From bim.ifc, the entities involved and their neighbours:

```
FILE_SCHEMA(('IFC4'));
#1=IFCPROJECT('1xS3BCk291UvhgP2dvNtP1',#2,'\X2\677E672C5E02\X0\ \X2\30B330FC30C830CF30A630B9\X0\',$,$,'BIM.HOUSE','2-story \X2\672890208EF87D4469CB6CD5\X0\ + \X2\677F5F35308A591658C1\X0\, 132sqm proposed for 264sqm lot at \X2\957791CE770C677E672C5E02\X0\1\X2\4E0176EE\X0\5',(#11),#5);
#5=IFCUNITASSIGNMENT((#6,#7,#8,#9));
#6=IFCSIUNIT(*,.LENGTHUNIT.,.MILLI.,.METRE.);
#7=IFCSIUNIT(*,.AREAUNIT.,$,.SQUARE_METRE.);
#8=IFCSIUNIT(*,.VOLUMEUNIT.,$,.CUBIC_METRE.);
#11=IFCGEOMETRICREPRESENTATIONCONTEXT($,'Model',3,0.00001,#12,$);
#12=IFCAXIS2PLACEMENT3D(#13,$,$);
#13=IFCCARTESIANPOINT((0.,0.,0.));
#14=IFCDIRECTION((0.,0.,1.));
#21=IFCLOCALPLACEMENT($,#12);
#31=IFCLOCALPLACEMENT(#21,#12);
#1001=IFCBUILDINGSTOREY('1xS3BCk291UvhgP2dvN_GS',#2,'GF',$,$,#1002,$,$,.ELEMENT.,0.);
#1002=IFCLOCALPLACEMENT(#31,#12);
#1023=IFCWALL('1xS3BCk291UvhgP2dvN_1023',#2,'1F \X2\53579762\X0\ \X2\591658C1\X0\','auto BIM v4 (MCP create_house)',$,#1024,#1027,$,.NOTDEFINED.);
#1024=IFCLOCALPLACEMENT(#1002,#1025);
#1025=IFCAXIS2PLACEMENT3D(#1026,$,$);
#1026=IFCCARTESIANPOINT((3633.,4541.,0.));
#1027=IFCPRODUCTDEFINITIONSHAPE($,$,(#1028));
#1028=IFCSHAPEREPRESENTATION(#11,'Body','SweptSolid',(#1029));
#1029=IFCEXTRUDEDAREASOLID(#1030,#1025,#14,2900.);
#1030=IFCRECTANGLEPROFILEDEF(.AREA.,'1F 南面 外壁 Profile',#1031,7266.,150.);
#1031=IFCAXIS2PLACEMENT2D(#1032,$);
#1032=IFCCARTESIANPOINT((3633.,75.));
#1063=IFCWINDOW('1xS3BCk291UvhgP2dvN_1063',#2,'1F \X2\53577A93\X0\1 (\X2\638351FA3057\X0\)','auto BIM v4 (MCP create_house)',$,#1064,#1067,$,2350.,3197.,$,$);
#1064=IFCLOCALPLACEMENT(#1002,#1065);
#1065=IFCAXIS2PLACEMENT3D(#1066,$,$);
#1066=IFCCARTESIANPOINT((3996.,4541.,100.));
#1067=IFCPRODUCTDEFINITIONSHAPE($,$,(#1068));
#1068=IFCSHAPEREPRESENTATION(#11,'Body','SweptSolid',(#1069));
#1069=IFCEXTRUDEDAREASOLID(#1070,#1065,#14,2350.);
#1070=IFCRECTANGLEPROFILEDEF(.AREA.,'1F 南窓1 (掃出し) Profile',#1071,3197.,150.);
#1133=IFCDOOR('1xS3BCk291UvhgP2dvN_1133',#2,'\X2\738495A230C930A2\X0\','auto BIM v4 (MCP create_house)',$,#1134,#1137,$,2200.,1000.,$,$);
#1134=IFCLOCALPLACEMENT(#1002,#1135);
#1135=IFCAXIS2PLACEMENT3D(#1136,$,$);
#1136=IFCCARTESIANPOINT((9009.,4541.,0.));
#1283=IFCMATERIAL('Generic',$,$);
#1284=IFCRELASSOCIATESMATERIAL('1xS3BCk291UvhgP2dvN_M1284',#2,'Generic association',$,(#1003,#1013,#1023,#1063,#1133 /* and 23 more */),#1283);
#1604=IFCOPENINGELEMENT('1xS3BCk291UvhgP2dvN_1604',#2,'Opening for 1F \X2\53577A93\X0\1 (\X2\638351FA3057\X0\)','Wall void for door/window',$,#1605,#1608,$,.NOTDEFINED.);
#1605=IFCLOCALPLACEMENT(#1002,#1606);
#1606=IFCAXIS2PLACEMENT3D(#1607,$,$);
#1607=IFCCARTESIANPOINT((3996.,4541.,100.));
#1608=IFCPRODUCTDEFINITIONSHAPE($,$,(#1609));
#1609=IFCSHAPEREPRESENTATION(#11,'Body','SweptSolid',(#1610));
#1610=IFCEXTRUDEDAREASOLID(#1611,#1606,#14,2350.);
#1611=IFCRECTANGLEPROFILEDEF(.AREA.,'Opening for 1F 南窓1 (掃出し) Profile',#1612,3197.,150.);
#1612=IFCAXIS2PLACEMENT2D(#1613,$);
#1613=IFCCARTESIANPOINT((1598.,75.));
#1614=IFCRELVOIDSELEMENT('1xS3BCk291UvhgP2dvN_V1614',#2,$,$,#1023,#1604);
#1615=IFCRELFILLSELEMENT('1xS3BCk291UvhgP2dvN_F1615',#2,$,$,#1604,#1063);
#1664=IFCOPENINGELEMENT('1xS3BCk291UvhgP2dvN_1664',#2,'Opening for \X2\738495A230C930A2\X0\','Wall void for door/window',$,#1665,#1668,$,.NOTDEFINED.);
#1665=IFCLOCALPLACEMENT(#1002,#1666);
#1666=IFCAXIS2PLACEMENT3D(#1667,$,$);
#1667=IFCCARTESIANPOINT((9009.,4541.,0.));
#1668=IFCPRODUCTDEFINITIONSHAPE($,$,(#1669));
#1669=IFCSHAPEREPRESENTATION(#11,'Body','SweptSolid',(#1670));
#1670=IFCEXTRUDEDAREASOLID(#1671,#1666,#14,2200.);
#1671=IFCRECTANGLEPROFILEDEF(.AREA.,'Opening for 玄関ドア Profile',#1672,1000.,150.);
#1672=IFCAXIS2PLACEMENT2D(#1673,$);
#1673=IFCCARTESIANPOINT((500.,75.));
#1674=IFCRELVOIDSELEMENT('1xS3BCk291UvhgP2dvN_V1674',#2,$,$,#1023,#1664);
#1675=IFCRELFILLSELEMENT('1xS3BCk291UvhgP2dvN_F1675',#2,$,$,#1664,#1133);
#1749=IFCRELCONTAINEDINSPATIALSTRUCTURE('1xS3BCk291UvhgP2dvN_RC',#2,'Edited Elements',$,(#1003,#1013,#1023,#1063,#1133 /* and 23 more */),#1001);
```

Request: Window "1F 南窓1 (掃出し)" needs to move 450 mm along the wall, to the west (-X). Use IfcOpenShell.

```python
import ifcopenshell
import ifcopenshell.api.geometry
import ifcopenshell.util.placement
import ifcopenshell.util.unit

model = ifcopenshell.open("bim.ifc")
unit_scale = ifcopenshell.util.unit.calculate_unit_scale(model)

window = model.by_id(1063)
opening = window.FillsVoids[0].RelatingOpeningElement
wall = opening.VoidsElements[0].RelatingBuildingElement

wall_matrix = ifcopenshell.util.placement.get_local_placement(wall.ObjectPlacement)
shift = wall_matrix[:3, 0] * -0.45 / unit_scale
before = ifcopenshell.util.placement.get_local_placement(window.ObjectPlacement)[:3, 3].copy()

# The window is not placed relative to its opening, so move both.
for product in (opening, window):
    matrix = ifcopenshell.util.placement.get_local_placement(product.ObjectPlacement)
    matrix[:3, 3] += shift
    ifcopenshell.api.geometry.edit_object_placement(model, product=product, matrix=matrix, is_si=False)

after = ifcopenshell.util.placement.get_local_placement(window.ObjectPlacement)[:3, 3]
print("window moved by", (after - before).round(3) + 0.0)

model.write("bim_rev.ifc")
```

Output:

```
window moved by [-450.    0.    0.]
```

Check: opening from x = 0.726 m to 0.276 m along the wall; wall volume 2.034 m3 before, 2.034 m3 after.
